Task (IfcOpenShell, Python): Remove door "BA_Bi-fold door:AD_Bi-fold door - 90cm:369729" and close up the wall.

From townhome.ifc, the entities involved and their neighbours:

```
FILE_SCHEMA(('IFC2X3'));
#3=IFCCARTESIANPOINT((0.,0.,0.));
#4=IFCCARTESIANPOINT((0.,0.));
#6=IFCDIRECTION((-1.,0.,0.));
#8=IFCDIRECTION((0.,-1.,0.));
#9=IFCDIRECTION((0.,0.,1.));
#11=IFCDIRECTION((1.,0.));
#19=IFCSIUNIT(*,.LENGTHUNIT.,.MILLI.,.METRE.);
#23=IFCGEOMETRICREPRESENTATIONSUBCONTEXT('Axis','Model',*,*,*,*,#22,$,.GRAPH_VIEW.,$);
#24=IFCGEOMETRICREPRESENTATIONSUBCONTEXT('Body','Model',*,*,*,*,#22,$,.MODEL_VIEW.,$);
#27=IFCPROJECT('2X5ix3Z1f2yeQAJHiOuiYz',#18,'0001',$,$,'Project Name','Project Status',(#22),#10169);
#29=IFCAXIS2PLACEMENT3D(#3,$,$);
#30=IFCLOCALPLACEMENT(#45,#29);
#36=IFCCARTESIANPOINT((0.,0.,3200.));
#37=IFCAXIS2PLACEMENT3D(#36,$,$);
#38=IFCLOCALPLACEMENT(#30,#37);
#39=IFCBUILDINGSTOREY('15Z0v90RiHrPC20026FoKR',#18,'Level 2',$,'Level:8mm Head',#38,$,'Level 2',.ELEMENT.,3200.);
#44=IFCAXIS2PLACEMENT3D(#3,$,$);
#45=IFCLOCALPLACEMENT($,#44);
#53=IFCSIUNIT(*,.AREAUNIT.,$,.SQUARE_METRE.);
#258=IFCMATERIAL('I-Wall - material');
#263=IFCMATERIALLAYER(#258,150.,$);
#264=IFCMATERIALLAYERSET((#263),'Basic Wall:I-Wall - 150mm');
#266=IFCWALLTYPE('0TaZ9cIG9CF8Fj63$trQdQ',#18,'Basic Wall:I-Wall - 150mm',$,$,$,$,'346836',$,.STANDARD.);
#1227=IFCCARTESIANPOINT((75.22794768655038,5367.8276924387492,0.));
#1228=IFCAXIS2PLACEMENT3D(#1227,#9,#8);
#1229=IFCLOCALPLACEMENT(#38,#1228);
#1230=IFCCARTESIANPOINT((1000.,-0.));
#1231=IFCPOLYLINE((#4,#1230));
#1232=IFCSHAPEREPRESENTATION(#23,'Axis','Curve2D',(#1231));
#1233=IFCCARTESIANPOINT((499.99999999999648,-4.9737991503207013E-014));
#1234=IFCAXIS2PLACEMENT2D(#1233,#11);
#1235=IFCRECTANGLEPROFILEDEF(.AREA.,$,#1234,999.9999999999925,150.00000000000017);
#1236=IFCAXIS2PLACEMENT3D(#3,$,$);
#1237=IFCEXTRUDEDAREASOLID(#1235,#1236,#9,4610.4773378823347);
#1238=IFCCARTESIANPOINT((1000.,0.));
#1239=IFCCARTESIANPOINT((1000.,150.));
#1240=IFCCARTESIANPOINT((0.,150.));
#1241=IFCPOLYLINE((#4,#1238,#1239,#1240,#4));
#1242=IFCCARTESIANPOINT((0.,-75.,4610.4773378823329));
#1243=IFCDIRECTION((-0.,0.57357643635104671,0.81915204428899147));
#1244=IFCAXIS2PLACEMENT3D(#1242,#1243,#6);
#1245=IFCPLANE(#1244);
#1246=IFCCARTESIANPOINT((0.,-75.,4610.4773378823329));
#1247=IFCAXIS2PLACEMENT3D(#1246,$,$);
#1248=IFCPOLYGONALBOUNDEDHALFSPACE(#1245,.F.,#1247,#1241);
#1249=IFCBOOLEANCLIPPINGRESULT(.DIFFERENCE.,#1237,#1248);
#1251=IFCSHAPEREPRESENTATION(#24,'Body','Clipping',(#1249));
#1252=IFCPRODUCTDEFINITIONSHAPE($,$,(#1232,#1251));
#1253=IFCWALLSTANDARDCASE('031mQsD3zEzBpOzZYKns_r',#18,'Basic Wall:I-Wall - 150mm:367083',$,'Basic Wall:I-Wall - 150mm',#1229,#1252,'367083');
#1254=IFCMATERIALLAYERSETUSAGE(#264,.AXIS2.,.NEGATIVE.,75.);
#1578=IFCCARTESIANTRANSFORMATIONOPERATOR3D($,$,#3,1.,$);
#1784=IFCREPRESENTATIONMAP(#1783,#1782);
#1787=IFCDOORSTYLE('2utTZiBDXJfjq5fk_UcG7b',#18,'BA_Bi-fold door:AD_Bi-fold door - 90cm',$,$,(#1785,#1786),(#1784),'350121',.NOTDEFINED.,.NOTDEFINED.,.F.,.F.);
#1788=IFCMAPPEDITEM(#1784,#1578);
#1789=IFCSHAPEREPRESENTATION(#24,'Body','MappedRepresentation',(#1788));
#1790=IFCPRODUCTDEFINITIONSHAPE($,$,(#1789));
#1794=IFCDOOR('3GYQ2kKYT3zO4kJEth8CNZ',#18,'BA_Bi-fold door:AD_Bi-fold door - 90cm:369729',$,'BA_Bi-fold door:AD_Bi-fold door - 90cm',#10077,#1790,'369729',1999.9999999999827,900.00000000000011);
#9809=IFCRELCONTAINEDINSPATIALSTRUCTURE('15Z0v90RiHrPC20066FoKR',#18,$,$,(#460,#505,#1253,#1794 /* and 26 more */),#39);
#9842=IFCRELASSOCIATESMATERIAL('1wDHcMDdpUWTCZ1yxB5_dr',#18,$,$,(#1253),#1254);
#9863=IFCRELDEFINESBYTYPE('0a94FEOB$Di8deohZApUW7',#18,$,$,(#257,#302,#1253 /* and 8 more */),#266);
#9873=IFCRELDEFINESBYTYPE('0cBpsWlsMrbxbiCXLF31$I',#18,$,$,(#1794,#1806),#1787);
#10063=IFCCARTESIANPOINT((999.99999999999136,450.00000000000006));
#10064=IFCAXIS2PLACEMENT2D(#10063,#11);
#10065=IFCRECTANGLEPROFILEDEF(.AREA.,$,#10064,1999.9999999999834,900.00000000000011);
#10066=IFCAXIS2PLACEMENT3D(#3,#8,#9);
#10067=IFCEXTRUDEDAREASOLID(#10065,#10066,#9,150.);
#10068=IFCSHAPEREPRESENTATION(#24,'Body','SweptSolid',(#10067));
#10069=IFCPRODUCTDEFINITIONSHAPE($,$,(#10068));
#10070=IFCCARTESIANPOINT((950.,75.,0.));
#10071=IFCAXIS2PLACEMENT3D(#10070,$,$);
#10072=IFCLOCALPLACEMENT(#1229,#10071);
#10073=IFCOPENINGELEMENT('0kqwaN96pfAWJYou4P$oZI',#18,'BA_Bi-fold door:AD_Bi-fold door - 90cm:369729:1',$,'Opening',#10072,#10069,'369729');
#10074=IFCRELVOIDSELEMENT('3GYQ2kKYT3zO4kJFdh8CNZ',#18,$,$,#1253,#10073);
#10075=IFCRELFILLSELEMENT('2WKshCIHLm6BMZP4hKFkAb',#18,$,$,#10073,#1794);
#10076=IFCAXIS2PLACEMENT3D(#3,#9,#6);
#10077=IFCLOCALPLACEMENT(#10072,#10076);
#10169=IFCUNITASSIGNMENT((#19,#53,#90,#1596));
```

```python
import ifcopenshell
import ifcopenshell.api.feature
import ifcopenshell.api.root
import ifcopenshell.geom
import ifcopenshell.util.shape

model = ifcopenshell.open("townhome.ifc")
settings = ifcopenshell.geom.settings()


def volume(element):
    """Net volume in cubic metres, openings subtracted."""
    shape = ifcopenshell.geom.create_shape(settings, element)
    return ifcopenshell.util.shape.get_volume(shape.geometry)


door = model.by_id(1794)
opening = door.FillsVoids[0].RelatingOpeningElement
wall = opening.VoidsElements[0].RelatingBuildingElement
before = volume(wall)

ifcopenshell.api.root.remove_product(model, product=door)
ifcopenshell.api.feature.remove_feature(model, feature=opening)

after = volume(wall)

print(f"wall volume {before:.3f} -> {after:.3f} m3")

model.write("townhome_edited.ifc")
```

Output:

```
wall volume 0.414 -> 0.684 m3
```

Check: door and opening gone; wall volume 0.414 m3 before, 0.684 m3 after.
